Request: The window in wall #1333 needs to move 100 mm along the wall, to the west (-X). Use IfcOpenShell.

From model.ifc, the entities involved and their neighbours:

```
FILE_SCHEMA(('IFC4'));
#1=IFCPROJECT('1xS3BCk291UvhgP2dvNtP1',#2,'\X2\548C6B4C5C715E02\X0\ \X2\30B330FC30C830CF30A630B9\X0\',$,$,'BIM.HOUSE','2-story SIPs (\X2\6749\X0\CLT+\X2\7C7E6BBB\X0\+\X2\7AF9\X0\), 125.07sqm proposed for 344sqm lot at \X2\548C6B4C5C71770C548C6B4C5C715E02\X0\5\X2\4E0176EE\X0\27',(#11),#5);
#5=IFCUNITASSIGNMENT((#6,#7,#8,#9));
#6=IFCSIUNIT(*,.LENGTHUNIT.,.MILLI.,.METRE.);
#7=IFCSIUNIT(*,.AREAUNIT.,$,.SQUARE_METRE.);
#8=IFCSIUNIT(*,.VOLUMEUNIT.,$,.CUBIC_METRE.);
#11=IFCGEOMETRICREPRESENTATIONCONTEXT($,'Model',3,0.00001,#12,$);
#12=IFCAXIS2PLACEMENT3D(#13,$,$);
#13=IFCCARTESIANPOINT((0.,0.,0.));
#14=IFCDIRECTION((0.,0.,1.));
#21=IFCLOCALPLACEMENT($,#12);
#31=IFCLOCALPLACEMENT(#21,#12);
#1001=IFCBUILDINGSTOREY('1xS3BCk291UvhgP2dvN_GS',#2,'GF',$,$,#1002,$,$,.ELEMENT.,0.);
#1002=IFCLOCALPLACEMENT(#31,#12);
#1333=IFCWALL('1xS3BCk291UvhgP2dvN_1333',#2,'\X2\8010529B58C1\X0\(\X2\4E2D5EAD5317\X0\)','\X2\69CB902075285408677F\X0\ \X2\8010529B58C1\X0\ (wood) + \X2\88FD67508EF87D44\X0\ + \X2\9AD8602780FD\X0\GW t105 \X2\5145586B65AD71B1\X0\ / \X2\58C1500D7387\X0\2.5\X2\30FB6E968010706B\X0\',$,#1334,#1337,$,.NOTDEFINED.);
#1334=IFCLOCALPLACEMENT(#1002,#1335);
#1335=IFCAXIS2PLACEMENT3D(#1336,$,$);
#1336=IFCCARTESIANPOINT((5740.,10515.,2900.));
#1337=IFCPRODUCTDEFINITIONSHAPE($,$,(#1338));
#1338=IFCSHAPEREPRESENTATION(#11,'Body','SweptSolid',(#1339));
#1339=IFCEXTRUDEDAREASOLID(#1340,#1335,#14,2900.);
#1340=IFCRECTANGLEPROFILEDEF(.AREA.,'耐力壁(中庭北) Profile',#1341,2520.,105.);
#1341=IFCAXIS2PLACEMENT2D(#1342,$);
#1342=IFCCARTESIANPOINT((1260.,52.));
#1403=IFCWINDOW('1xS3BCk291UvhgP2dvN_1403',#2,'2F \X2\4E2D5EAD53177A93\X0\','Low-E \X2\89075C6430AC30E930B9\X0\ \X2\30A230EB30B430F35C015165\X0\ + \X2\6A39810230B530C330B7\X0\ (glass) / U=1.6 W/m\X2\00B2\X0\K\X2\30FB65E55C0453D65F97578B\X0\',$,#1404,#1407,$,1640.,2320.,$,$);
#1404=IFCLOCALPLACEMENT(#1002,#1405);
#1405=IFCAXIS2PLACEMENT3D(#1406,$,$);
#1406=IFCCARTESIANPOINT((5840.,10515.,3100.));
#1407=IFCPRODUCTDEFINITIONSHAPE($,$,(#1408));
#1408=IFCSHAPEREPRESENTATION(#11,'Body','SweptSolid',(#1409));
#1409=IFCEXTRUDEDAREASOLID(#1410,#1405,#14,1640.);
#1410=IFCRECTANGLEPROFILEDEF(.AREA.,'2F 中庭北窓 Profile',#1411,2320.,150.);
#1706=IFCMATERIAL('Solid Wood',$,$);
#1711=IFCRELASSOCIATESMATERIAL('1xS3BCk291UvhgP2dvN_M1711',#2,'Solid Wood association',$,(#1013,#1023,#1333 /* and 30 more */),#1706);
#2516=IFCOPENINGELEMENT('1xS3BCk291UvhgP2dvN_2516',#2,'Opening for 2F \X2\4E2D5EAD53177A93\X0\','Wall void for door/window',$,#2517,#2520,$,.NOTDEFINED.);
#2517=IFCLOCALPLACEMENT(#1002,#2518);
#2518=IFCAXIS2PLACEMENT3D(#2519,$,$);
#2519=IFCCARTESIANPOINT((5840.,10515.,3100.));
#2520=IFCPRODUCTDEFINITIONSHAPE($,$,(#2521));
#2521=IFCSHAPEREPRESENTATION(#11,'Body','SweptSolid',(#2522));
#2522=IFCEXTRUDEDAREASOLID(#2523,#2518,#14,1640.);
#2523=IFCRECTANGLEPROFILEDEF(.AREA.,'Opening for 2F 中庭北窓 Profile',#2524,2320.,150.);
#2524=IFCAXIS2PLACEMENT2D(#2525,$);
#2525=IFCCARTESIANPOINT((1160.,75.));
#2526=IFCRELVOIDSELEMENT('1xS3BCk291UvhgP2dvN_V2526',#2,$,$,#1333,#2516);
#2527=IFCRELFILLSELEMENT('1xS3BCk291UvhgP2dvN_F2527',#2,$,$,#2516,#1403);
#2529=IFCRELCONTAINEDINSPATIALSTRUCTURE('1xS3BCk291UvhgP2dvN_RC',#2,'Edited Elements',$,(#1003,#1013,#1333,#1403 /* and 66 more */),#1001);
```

```python
import ifcopenshell
import ifcopenshell.api.geometry
import ifcopenshell.util.placement
import ifcopenshell.util.unit

model = ifcopenshell.open("model.ifc")
unit_scale = ifcopenshell.util.unit.calculate_unit_scale(model)

window = model.by_guid("1xS3BCk291UvhgP2dvN_1403")
opening = window.FillsVoids[0].RelatingOpeningElement
wall = opening.VoidsElements[0].RelatingBuildingElement

wall_matrix = ifcopenshell.util.placement.get_local_placement(wall.ObjectPlacement)
shift = wall_matrix[:3, 0] * -0.1 / unit_scale
before = ifcopenshell.util.placement.get_local_placement(window.ObjectPlacement)[:3, 3].copy()

# The window is not placed relative to its opening, so move both.
for product in (opening, window):
    matrix = ifcopenshell.util.placement.get_local_placement(product.ObjectPlacement)
    matrix[:3, 3] += shift
    ifcopenshell.api.geometry.edit_object_placement(model, product=product, matrix=matrix, is_si=False)

after = ifcopenshell.util.placement.get_local_placement(window.ObjectPlacement)[:3, 3]
print("window moved by", (after - before).round(3) + 0.0)

model.write("model_v2.ifc")
```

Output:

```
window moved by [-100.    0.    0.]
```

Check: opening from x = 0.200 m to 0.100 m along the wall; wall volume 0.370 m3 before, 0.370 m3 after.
